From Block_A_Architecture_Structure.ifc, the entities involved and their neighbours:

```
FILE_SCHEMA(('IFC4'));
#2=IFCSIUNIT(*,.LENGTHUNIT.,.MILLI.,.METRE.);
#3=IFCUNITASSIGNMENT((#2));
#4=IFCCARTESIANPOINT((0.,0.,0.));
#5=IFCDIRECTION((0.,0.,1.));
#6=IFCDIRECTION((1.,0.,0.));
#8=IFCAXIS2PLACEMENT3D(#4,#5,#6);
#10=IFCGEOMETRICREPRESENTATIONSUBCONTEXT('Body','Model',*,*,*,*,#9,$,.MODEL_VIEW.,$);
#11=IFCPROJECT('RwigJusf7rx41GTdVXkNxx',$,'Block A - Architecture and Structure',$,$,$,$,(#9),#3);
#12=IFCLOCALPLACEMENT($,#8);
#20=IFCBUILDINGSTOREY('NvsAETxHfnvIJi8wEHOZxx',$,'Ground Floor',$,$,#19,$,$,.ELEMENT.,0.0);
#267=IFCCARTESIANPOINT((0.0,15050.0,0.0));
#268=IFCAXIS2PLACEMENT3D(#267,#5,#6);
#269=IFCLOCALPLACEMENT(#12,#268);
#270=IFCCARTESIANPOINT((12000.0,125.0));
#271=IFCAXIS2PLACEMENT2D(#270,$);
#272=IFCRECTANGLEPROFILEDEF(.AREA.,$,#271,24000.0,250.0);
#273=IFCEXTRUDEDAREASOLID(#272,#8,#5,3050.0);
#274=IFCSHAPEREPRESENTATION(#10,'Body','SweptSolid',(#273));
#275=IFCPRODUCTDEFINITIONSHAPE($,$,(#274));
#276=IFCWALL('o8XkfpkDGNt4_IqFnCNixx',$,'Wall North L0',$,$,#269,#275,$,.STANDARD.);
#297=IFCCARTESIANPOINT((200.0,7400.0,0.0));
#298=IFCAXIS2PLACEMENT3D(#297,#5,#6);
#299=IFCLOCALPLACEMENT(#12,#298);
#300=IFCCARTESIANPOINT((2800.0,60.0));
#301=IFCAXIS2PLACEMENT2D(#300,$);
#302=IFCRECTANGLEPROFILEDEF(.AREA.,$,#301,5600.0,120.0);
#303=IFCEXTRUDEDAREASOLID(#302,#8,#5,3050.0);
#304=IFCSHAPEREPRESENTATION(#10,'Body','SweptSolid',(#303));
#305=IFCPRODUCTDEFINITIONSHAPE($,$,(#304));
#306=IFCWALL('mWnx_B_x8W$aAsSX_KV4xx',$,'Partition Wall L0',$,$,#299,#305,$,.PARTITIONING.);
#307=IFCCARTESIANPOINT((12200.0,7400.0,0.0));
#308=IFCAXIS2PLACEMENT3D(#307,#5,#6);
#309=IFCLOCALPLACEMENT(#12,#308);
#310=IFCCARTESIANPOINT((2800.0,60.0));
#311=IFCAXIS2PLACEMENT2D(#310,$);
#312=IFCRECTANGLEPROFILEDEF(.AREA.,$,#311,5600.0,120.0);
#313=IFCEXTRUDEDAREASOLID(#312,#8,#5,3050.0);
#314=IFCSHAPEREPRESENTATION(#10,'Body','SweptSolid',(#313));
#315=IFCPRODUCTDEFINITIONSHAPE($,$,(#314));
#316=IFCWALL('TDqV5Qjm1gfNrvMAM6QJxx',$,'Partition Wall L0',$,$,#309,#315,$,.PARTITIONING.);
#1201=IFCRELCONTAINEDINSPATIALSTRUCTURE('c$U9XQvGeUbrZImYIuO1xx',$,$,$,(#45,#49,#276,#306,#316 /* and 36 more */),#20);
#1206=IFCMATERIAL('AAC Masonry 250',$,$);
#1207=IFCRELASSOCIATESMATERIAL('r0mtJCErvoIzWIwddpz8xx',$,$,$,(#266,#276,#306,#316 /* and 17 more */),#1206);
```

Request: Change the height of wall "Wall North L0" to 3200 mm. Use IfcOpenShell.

```python
import ifcopenshell
import ifcopenshell.geom
import ifcopenshell.util.representation
import ifcopenshell.util.shape

model = ifcopenshell.open("Block_A_Architecture_Structure.ifc")
settings = ifcopenshell.geom.settings()


def volume(element):
    """Net volume in cubic metres, openings subtracted."""
    shape = ifcopenshell.geom.create_shape(settings, element)
    return ifcopenshell.util.shape.get_volume(shape.geometry)


wall = model.by_guid("o8XkfpkDGNt4_IqFnCNixx")
before = volume(wall)

body = ifcopenshell.util.representation.get_representation(wall, "Model", "Body")
solid = body.Items[0]
old_height = solid.Depth
solid.Depth = 3200.0
after = volume(wall)

print(f"height {old_height:g} -> {solid.Depth:g}, volume {before:.3f} -> {after:.3f} m3")

model.write("Block_A_Architecture_Structure_v2.ifc")
```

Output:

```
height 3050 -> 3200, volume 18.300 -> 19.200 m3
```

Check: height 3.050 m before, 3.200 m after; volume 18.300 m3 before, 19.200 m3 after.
